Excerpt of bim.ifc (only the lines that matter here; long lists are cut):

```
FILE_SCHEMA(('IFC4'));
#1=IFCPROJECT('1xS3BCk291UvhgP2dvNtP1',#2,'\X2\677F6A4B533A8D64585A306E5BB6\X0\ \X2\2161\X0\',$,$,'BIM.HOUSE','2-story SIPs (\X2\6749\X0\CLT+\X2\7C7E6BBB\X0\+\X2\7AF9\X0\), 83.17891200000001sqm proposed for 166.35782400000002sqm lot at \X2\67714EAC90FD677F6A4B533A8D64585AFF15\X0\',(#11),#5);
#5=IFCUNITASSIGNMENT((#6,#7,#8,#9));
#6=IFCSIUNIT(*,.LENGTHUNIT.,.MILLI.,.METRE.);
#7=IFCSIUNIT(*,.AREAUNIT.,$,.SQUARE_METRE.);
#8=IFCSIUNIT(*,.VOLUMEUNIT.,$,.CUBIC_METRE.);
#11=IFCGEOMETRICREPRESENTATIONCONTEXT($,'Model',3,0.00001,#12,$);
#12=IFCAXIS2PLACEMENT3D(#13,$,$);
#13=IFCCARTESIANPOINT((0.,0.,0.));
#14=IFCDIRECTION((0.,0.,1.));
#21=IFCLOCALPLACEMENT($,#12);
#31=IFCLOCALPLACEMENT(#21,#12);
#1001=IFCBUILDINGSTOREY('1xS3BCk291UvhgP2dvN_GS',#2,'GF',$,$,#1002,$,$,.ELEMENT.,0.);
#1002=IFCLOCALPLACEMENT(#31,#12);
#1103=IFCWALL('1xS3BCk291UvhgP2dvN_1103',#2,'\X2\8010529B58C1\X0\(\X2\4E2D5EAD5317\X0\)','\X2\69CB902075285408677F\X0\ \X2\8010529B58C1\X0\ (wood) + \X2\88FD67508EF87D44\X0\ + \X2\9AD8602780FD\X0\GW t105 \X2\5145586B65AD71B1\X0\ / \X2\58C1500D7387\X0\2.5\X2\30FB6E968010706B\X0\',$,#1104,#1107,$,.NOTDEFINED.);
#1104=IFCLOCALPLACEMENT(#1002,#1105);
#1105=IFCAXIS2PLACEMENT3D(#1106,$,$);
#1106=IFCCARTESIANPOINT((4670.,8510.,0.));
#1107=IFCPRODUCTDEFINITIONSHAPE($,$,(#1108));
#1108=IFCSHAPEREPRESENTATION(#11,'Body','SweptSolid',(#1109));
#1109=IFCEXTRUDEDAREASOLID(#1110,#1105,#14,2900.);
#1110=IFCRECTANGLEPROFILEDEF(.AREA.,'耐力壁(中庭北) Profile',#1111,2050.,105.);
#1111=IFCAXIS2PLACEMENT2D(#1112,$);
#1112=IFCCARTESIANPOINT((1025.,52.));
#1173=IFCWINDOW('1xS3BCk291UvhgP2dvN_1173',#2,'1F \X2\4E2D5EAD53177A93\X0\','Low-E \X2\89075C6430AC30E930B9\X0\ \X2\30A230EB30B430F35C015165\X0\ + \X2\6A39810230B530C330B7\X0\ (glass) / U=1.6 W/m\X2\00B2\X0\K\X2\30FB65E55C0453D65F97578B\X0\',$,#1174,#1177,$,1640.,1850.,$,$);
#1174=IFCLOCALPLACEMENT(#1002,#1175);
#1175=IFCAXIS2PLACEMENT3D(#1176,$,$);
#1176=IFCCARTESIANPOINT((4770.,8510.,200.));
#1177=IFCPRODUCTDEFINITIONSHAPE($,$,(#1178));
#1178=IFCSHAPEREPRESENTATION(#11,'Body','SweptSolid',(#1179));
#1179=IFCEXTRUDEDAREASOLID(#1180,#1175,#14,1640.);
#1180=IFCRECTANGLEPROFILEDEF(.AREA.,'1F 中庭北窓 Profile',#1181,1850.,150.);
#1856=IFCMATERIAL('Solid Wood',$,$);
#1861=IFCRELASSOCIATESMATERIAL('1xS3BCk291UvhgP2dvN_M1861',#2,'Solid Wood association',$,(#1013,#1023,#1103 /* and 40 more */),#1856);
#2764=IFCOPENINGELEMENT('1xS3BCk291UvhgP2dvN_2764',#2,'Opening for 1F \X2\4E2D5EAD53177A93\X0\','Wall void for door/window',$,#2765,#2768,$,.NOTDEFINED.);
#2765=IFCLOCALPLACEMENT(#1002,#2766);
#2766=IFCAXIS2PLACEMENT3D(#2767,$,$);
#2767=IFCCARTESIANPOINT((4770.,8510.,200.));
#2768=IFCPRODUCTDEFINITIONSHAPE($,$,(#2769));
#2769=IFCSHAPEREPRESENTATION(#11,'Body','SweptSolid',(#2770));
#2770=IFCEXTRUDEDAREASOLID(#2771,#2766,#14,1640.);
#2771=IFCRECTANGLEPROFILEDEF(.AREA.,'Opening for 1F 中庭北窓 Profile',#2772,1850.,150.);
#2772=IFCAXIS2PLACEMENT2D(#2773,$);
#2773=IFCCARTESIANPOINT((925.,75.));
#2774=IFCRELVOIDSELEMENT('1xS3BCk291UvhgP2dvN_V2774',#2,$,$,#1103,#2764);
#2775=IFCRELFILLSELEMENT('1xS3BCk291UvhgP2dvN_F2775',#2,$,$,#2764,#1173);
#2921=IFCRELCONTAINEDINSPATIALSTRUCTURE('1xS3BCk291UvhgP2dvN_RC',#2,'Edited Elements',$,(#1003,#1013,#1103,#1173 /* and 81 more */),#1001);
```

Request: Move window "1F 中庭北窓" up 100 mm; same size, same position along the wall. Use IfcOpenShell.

```python
import numpy as np
import ifcopenshell
import ifcopenshell.api.geometry
import ifcopenshell.util.placement
import ifcopenshell.util.unit

model = ifcopenshell.open("bim.ifc")
unit_scale = ifcopenshell.util.unit.calculate_unit_scale(model)

window = model.by_guid("1xS3BCk291UvhgP2dvN_1173")
opening = window.FillsVoids[0].RelatingOpeningElement
dz = 0.1 / unit_scale

shift = np.array([0.0, 0.0, dz])
# The window is not placed relative to its opening, so move both.
for product in (opening, window):
    matrix = ifcopenshell.util.placement.get_local_placement(product.ObjectPlacement)
    matrix[:3, 3] += shift
    ifcopenshell.api.geometry.edit_object_placement(model, product=product, matrix=matrix, is_si=False)

print(f"moved by {dz * unit_scale:+.3f} m")

model.write("bim_updated.ifc")
```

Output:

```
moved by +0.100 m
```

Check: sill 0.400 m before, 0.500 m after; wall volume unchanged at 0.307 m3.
